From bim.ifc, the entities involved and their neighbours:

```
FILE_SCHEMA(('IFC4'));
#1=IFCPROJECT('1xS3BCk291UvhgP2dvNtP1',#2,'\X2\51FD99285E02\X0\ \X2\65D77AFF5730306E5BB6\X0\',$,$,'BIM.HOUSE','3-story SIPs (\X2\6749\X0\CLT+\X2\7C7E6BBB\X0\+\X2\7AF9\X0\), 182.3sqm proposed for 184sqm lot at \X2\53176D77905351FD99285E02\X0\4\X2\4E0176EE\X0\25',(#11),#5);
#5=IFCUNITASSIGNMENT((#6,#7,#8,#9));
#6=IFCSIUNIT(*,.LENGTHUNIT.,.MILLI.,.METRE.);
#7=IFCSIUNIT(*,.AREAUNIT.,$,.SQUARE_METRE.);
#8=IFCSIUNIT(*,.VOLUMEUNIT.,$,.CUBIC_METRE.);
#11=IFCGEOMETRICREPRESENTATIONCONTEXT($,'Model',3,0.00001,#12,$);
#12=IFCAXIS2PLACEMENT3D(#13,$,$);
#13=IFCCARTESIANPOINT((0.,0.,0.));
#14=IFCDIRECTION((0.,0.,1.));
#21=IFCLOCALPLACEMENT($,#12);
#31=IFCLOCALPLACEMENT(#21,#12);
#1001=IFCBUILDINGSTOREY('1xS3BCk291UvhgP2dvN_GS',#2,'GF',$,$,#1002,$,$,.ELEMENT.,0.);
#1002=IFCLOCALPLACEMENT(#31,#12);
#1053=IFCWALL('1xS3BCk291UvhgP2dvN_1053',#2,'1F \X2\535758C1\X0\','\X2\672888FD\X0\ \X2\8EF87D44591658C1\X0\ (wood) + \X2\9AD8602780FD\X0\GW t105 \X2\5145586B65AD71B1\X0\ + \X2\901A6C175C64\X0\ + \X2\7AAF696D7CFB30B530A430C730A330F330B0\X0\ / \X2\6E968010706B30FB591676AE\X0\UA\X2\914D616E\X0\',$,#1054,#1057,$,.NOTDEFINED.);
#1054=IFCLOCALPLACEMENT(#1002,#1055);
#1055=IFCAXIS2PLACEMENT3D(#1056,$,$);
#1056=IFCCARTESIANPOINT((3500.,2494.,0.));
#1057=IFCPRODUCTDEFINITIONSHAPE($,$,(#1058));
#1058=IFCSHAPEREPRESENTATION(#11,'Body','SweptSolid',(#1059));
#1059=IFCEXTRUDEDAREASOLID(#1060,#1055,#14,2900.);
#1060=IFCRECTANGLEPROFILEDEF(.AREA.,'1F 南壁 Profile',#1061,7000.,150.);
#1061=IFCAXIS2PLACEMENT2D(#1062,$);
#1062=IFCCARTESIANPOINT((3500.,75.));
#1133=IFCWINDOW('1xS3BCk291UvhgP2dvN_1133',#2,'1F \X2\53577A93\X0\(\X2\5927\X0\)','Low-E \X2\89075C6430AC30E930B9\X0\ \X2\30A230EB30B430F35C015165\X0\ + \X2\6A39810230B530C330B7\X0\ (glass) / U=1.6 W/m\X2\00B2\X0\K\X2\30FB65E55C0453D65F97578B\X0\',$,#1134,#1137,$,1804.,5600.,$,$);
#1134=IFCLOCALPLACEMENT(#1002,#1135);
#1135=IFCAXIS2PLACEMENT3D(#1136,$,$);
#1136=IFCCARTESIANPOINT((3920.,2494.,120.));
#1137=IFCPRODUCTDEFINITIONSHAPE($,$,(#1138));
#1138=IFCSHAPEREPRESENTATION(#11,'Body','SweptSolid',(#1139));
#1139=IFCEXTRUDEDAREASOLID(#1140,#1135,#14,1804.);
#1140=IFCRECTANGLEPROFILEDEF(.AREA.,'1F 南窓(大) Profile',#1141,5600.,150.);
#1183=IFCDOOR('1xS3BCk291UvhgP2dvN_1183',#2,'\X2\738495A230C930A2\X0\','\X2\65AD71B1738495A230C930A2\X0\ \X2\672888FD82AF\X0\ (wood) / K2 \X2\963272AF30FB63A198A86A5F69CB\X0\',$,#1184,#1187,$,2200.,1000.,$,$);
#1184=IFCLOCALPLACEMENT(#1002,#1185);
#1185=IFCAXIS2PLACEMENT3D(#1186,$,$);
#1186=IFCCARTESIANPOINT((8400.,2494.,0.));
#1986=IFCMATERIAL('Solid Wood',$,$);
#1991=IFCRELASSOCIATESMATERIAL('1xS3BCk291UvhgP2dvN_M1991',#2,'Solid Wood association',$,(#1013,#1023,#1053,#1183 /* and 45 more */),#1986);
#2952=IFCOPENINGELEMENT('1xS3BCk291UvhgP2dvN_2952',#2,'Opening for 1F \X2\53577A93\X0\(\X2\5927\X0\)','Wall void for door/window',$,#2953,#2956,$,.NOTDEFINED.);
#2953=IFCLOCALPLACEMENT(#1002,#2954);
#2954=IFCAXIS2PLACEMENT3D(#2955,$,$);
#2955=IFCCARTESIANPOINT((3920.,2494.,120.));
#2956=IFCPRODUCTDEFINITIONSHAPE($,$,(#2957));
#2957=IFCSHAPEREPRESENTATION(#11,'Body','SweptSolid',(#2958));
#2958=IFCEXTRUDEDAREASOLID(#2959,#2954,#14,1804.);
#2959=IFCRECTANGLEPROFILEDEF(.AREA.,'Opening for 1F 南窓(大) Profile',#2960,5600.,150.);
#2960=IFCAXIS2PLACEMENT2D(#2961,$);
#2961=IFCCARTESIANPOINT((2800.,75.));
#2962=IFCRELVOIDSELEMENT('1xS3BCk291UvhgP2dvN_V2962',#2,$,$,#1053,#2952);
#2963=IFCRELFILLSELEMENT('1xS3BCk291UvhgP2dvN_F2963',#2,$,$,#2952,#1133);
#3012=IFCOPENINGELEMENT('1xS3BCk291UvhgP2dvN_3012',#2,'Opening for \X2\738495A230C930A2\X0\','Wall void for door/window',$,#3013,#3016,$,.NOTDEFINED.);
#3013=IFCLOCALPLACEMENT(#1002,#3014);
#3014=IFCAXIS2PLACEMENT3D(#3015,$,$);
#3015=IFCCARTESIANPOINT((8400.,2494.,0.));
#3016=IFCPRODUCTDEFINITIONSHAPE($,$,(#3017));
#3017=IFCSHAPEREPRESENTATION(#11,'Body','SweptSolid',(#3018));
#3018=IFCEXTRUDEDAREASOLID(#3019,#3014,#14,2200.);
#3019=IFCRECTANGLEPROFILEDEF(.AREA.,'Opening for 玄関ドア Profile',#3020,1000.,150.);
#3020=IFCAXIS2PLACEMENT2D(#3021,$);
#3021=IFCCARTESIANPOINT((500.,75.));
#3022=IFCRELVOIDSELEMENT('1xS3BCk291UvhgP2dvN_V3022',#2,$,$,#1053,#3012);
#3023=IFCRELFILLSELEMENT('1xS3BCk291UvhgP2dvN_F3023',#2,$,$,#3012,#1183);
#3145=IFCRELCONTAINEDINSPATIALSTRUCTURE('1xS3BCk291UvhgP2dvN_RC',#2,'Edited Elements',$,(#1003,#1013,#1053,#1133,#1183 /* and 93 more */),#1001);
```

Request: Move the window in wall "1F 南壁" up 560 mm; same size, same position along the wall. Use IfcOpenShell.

```python
import numpy as np
import ifcopenshell
import ifcopenshell.api.geometry
import ifcopenshell.util.placement
import ifcopenshell.util.unit

model = ifcopenshell.open("bim.ifc")
unit_scale = ifcopenshell.util.unit.calculate_unit_scale(model)

window = model.by_guid("1xS3BCk291UvhgP2dvN_1133")
opening = window.FillsVoids[0].RelatingOpeningElement
dz = 560.0

shift = np.array([0.0, 0.0, dz])
# The window is not placed relative to its opening, so move both.
for product in (opening, window):
    matrix = ifcopenshell.util.placement.get_local_placement(product.ObjectPlacement)
    matrix[:3, 3] += shift
    ifcopenshell.api.geometry.edit_object_placement(model, product=product, matrix=matrix, is_si=False)

print(f"moved by {dz * unit_scale:+.3f} m")

model.write("bim_updated.ifc")
```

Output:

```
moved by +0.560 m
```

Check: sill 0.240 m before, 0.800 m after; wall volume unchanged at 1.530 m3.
